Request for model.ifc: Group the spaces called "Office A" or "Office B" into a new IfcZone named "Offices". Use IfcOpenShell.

First a look at what the model holds.

```python
import ifcopenshell

model = ifcopenshell.open("model.ifc")
print(model.schema)
seen = {}
for space in model.by_type("IfcSpace"):
    seen[space.LongName] = seen.get(space.LongName, 0) + 1
for name, count in sorted(seen.items(), key=str):
    print(count, "x", name)
print("zones:", [z.Name for z in model.by_type("IfcZone")][:20])
```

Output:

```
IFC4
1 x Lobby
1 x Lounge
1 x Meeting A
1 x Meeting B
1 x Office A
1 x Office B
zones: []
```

```python
import ifcopenshell
import ifcopenshell.api.group
import ifcopenshell.api.root

model = ifcopenshell.open("model.ifc")

names = {"Office A", "Office B"}
spaces = [s for s in model.by_type("IfcSpace") if s.LongName in names]

zone = ifcopenshell.api.root.create_entity(model, ifc_class="IfcZone", name="Offices")
ifcopenshell.api.group.assign_group(model, products=spaces, group=zone)
print(len(spaces), "spaces in", zone.Name)

model.write("model_v2.ifc")
```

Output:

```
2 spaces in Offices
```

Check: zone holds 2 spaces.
